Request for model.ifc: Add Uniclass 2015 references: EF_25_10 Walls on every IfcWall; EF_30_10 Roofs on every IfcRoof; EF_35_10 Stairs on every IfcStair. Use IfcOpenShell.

First a look at what the model holds.

```python
import ifcopenshell

model = ifcopenshell.open("model.ifc")
print(model.schema)
print("classifications:", [c.Name for c in model.by_type("IfcClassification")])
for ifc_class in ("IfcDoor", "IfcRoof", "IfcStair", "IfcWall", "IfcWindow"):
    print(ifc_class, len(model.by_type(ifc_class)))
```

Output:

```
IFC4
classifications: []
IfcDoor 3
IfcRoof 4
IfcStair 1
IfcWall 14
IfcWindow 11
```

```python
import ifcopenshell
import ifcopenshell.api.classification

model = ifcopenshell.open("model.ifc")

system = ifcopenshell.api.classification.add_classification(model, classification="Uniclass 2015")

codes = {
    "IfcWall": ("EF_25_10", "Walls"),
    "IfcRoof": ("EF_30_10", "Roofs"),
    "IfcStair": ("EF_35_10", "Stairs"),
}
for ifc_class, (code, name) in codes.items():
    products = model.by_type(ifc_class)
    ifcopenshell.api.classification.add_reference(
        model, products=products, classification=system, identification=code, name=name
    )
    print(code, len(products))

model.write("model_edited.ifc")
```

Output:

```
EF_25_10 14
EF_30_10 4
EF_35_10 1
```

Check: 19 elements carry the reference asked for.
